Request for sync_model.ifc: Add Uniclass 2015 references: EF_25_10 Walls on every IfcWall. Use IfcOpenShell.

First a look at what the model holds.

```python
import ifcopenshell

model = ifcopenshell.open("sync_model.ifc")
print(model.schema)
print("classifications:", [c.Name for c in model.by_type("IfcClassification")])
for ifc_class in ("IfcDoor", "IfcRoof", "IfcStair", "IfcWall", "IfcWindow"):
    print(ifc_class, len(model.by_type(ifc_class)))
```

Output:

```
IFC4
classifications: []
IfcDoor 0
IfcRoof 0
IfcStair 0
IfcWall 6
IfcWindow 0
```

```python
import ifcopenshell
import ifcopenshell.api.classification

model = ifcopenshell.open("sync_model.ifc")

system = ifcopenshell.api.classification.add_classification(model, classification="Uniclass 2015")

codes = {
    "IfcWall": ("EF_25_10", "Walls"),
}
for ifc_class, (code, name) in codes.items():
    products = model.by_type(ifc_class)
    ifcopenshell.api.classification.add_reference(
        model, products=products, classification=system, identification=code, name=name
    )
    print(code, len(products))

model.write("sync_model_rev.ifc")
```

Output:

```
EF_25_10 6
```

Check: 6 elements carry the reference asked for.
